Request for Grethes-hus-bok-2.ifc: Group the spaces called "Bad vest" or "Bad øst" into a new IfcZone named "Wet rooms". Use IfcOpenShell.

First a look at what the model holds.

```python
import ifcopenshell

model = ifcopenshell.open("Grethes-hus-bok-2.ifc")
print(model.schema)
seen = {}
for space in model.by_type("IfcSpace"):
    seen[space.LongName] = seen.get(space.LongName, 0) + 1
for name, count in sorted(seen.items(), key=str):
    print(count, "x", name)
print("zones:", [z.Name for z in model.by_type("IfcZone")][:20])
```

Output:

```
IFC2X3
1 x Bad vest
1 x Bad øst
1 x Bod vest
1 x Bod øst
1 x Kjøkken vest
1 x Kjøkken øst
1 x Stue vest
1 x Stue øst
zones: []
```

```python
import ifcopenshell
import ifcopenshell.api.group
import ifcopenshell.api.root

model = ifcopenshell.open("Grethes-hus-bok-2.ifc")

names = {"Bad vest", "Bad øst"}
spaces = [s for s in model.by_type("IfcSpace") if s.LongName in names]

zone = ifcopenshell.api.root.create_entity(model, ifc_class="IfcZone", name="Wet rooms")
ifcopenshell.api.group.assign_group(model, products=spaces, group=zone)
print(len(spaces), "spaces in", zone.Name)

model.write("Grethes-hus-bok-2_rev.ifc")
```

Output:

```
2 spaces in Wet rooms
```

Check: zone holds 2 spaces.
